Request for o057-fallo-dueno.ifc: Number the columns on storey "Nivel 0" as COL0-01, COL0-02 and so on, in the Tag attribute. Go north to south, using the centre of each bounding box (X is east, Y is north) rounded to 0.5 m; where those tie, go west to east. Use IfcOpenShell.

First a look at what the model holds.

```python
import ifcopenshell
import ifcopenshell.util.element
import ifcopenshell.util.placement

model = ifcopenshell.open("o057-fallo-dueno.ifc")
print(model.schema)
storey = next(s for s in model.by_type("IfcBuildingStorey") if s.Name == "Nivel 0")
columns = [e for e in ifcopenshell.util.element.get_decomposition(storey) if e.is_a("IfcColumn")]
for e in sorted(columns, key=lambda e: e.id()):
    origin = ifcopenshell.util.placement.get_local_placement(e.ObjectPlacement)[:3, 3]
    print(e.id(), e.Tag, e.Name, origin.round(2) + 0.0, sep=" | ")
```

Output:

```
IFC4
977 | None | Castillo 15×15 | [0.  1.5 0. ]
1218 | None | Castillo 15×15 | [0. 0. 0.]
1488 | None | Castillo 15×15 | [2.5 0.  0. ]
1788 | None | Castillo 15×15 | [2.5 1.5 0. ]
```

```python
import ifcopenshell
import ifcopenshell.geom
import ifcopenshell.util.element
import ifcopenshell.util.shape

model = ifcopenshell.open("o057-fallo-dueno.ifc")
settings = ifcopenshell.geom.settings()
settings.set("use-world-coords", True)


def centre(element):
    shape = ifcopenshell.geom.create_shape(settings, element)
    return ifcopenshell.util.shape.get_bbox_centroid(shape.geometry)


storey = next(s for s in model.by_type("IfcBuildingStorey") if s.Name == "Nivel 0")
columns = [e for e in ifcopenshell.util.element.get_decomposition(storey) if e.is_a("IfcColumn")]

# Insertion points can sit at a corner or the storey origin, so sort by the geometry (in metres).
centres = {e: centre(e) for e in columns}
columns.sort(key=lambda e: (-round(centres[e][1] / 0.5), centres[e][0]))

for i, e in enumerate(columns, start=1):
    number = f"COL0-{i:02d}"
    e.Tag = number
    print(e.id(), number)

model.write("o057-fallo-dueno_rev.ifc")
```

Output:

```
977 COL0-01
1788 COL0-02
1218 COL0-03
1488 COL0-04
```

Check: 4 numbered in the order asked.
